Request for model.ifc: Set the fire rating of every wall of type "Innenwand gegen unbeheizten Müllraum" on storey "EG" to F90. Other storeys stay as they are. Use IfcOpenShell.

First a look at what the model holds.

```python
import ifcopenshell
import ifcopenshell.util.element

model = ifcopenshell.open("model.ifc")
print(model.schema)
storey = next(s for s in model.by_type("IfcBuildingStorey") if s.Name == "EG")
walls = [e for e in ifcopenshell.util.element.get_decomposition(storey) if e.is_a("IfcWall")]
seen = {}
for e in walls:
    element_type = ifcopenshell.util.element.get_type(e)
    key = (element_type.Name if element_type != e and element_type else None, ifcopenshell.util.element.get_pset(e, "Pset_WallCommon", "FireRating"))
    seen[key] = seen.get(key, 0) + 1
for (name, value), count in sorted(seen.items(), key=str):
    print(count, "x", name, "|", value)
```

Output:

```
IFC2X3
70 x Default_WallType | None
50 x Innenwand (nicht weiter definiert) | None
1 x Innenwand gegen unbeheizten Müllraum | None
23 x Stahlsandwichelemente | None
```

```python
import ifcopenshell
import ifcopenshell.api.pset
import ifcopenshell.util.element

model = ifcopenshell.open("model.ifc")

storey = next(s for s in model.by_type("IfcBuildingStorey") if s.Name == "EG")
walls = [e for e in ifcopenshell.util.element.get_decomposition(storey) if e.is_a("IfcWall")]

count = 0
for e in walls:
    element_type = ifcopenshell.util.element.get_type(e)
    if element_type in (None, e) or element_type.Name != "Innenwand gegen unbeheizten Müllraum":
        continue
    # add_pset returns the element's existing set when there is one.
    pset = ifcopenshell.api.pset.add_pset(model, product=e, name="Pset_WallCommon")
    ifcopenshell.api.pset.edit_pset(model, pset=pset, properties={"FireRating": "F90"})
    count += 1

print(count, "walls updated")

model.write("model_v2.ifc")
```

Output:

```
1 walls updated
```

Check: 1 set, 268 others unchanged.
